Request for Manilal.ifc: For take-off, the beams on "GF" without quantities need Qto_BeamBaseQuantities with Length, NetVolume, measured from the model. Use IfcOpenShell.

First a look at what the model holds.

```python
import ifcopenshell
import ifcopenshell.util.element
import ifcopenshell.util.unit

model = ifcopenshell.open("Manilal.ifc")
print(model.schema)
for unit_type in ("LENGTHUNIT", "AREAUNIT", "VOLUMEUNIT"):
    print(unit_type, ifcopenshell.util.unit.calculate_unit_scale(model, unit_type))
storey = next(s for s in model.by_type("IfcBuildingStorey") if s.Name == "GF")
beams = [e for e in ifcopenshell.util.element.get_decomposition(storey) if e.is_a("IfcBeam")]
for e in sorted(beams, key=lambda e: e.id()):
    print(e.id(), e.is_a(), e.Name, list(ifcopenshell.util.element.get_psets(e, qtos_only=True)), sep=" | ")
```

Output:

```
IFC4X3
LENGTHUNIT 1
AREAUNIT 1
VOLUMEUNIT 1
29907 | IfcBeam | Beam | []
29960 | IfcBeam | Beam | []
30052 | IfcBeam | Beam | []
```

```python
import ifcopenshell
import ifcopenshell.api.pset
import ifcopenshell.geom
import ifcopenshell.util.element
import ifcopenshell.util.shape
import ifcopenshell.util.unit

model = ifcopenshell.open("Manilal.ifc")
unit_scale = ifcopenshell.util.unit.calculate_unit_scale(model)
volume_scale = ifcopenshell.util.unit.calculate_unit_scale(model, "VOLUMEUNIT")
settings = ifcopenshell.geom.settings()

storey = next(s for s in model.by_type("IfcBuildingStorey") if s.Name == "GF")
beams = [e for e in ifcopenshell.util.element.get_decomposition(storey) if e.is_a("IfcBeam")]

for e in sorted(beams, key=lambda e: e.id()):
    if ifcopenshell.util.element.get_psets(e, qtos_only=True, should_inherit=False):
        continue
    # Geometry comes back in metres, in the element's own axes.
    shape = ifcopenshell.geom.create_shape(settings, e)
    values = {
        "Length": ifcopenshell.util.shape.get_max_xyz(shape.geometry) / unit_scale,
        "NetVolume": ifcopenshell.util.shape.get_volume(shape.geometry) / volume_scale,
    }
    qto = ifcopenshell.api.pset.add_qto(model, product=e, name="Qto_BeamBaseQuantities")
    ifcopenshell.api.pset.edit_qto(model, qto=qto, properties=values)
    print(e.id(), {k: round(v, 3) for k, v in values.items()})

model.write("Manilal_updated.ifc")
```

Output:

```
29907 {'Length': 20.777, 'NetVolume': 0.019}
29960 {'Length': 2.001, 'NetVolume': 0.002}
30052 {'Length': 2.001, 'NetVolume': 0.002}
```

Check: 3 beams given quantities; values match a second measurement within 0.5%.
